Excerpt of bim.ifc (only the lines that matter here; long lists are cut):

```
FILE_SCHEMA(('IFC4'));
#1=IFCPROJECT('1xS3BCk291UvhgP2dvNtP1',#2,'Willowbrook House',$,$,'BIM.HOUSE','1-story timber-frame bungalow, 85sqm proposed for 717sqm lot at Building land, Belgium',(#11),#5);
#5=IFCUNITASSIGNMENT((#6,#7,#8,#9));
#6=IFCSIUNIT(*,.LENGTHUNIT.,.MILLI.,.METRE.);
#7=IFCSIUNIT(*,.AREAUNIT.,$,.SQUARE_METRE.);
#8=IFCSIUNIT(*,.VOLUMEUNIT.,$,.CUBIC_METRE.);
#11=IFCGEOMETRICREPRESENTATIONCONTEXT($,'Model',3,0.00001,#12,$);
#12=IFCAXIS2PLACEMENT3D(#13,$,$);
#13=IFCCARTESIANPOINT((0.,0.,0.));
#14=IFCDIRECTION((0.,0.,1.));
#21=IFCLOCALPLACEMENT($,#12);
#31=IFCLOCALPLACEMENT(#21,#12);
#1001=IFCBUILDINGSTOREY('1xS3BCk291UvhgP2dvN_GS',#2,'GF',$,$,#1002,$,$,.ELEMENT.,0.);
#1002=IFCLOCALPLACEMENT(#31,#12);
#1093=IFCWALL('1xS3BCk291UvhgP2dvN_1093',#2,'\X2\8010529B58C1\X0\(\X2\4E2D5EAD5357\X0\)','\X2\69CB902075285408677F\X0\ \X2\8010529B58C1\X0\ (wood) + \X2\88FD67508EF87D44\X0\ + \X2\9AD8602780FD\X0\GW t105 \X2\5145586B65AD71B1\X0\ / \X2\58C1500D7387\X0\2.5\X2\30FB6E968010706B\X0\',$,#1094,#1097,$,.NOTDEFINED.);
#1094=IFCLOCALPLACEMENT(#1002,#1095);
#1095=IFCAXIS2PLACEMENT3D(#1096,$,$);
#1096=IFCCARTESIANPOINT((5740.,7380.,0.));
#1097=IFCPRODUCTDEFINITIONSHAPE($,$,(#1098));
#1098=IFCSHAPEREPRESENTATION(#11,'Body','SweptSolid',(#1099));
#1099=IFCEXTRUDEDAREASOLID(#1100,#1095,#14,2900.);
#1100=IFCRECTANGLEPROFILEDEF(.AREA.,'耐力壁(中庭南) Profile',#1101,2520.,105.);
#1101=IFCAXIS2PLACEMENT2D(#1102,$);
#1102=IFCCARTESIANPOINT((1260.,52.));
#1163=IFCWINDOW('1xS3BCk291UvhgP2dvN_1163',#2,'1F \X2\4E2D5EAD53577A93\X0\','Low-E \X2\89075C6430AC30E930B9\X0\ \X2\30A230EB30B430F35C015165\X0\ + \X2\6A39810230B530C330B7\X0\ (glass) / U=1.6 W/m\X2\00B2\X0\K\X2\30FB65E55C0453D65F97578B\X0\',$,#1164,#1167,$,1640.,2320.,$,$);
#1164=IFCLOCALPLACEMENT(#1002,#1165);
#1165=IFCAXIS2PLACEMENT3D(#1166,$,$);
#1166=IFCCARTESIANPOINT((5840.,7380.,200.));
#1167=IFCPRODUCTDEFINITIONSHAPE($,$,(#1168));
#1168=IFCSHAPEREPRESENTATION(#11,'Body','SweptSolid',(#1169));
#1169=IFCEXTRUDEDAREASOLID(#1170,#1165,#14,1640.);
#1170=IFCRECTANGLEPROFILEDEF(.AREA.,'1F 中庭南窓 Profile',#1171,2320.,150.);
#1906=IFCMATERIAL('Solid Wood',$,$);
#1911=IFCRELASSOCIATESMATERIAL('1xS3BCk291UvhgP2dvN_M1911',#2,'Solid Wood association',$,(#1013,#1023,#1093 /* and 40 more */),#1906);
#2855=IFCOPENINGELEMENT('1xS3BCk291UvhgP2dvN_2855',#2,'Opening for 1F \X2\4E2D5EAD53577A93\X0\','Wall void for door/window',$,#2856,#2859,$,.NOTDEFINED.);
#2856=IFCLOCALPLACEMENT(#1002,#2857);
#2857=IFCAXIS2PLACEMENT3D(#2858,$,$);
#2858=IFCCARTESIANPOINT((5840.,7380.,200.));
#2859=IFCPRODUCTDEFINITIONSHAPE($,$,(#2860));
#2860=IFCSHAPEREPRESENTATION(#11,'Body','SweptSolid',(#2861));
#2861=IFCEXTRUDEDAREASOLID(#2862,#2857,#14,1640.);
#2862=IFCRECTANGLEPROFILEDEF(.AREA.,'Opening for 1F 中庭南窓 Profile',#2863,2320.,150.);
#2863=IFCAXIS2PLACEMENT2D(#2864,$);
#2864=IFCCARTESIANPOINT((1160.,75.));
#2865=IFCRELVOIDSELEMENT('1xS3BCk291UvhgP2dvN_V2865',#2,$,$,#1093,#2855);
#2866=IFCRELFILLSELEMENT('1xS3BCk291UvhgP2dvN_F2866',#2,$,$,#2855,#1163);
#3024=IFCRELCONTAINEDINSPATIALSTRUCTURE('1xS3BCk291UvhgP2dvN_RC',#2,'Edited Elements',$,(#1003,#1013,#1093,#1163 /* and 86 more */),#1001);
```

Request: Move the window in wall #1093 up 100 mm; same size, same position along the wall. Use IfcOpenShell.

```python
import numpy as np
import ifcopenshell
import ifcopenshell.api.geometry
import ifcopenshell.util.placement
import ifcopenshell.util.unit

model = ifcopenshell.open("bim.ifc")
unit_scale = ifcopenshell.util.unit.calculate_unit_scale(model)

window = model.by_id(1163)
opening = window.FillsVoids[0].RelatingOpeningElement
dz = 0.1 / unit_scale

shift = np.array([0.0, 0.0, dz])
# The window is not placed relative to its opening, so move both.
for product in (opening, window):
    matrix = ifcopenshell.util.placement.get_local_placement(product.ObjectPlacement)
    matrix[:3, 3] += shift
    ifcopenshell.api.geometry.edit_object_placement(model, product=product, matrix=matrix, is_si=False)

print(f"moved by {dz * unit_scale:+.3f} m")

model.write("bim-out.ifc")
```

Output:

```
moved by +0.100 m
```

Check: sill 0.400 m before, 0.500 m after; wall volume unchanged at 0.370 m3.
